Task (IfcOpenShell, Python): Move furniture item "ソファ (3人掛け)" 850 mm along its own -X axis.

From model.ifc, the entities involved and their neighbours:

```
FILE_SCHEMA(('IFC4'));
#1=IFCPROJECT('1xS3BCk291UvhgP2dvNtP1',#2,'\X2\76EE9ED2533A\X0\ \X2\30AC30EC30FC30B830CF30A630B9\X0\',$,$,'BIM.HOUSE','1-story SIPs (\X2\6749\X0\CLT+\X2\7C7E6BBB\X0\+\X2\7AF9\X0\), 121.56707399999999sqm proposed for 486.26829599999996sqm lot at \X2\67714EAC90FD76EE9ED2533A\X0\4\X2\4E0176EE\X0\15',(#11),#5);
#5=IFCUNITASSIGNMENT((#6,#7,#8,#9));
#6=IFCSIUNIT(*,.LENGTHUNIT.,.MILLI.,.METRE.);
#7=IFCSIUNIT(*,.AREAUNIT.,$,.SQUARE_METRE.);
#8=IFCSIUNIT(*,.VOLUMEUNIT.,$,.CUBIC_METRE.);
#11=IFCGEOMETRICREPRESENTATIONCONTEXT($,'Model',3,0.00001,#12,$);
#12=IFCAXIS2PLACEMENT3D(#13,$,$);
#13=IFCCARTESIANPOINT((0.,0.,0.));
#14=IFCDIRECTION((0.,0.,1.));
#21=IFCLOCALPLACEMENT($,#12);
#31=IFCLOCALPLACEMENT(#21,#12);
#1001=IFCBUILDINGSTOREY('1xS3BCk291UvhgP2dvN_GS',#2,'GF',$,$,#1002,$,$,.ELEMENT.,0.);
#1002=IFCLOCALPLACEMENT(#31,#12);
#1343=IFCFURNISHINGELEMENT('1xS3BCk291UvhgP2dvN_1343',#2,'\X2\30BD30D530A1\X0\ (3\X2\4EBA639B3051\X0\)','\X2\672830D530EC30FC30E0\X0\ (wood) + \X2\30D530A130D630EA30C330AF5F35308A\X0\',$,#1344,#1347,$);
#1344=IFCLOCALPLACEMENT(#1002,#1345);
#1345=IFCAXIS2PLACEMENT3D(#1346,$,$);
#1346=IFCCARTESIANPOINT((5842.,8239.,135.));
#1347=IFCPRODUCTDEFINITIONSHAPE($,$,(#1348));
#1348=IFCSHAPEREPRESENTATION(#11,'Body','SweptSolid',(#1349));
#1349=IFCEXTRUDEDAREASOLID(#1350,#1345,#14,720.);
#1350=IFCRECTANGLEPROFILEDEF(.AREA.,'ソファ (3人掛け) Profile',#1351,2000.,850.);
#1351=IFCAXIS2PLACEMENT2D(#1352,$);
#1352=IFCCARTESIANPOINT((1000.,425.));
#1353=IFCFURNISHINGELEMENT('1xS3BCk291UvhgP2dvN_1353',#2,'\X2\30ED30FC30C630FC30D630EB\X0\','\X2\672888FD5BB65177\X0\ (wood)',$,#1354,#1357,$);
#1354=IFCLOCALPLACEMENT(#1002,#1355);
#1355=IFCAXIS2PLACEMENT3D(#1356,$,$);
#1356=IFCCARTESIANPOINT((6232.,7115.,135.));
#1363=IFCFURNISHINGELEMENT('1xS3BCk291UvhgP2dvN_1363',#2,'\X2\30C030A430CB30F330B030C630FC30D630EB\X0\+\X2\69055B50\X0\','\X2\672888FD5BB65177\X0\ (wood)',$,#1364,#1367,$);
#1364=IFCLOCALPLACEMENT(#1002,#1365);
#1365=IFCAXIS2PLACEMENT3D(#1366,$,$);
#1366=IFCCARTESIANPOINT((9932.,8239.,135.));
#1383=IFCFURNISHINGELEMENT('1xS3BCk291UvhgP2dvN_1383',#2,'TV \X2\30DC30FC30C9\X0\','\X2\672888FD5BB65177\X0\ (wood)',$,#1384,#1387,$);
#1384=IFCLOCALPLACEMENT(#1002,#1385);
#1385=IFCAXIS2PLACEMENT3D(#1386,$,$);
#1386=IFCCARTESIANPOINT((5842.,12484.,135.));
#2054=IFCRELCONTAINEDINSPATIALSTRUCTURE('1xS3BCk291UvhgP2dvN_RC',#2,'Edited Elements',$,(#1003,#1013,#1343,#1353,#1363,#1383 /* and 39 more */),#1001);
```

```python
import ifcopenshell
import ifcopenshell.api.geometry
import ifcopenshell.util.placement
import ifcopenshell.util.unit

model = ifcopenshell.open("model.ifc")
unit_scale = ifcopenshell.util.unit.calculate_unit_scale(model)

item = model.by_id(1343)
matrix = ifcopenshell.util.placement.get_local_placement(item.ObjectPlacement)
matrix[:3, 3] -= matrix[:3, 0] * 0.85 / unit_scale
ifcopenshell.api.geometry.edit_object_placement(model, product=item, matrix=matrix, is_si=False)

print(ifcopenshell.util.placement.get_local_placement(item.ObjectPlacement).round(3) + 0.0)

model.write("model_rev.ifc")
```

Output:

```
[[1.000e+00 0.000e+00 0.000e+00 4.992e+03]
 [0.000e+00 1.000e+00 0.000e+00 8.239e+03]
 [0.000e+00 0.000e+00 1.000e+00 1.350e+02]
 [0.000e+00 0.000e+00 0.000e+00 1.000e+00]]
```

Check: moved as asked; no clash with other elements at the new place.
